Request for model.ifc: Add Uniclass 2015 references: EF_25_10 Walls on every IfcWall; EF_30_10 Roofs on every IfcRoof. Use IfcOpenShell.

First a look at what the model holds.

```python
import ifcopenshell

model = ifcopenshell.open("model.ifc")
print(model.schema)
print("classifications:", [c.Name for c in model.by_type("IfcClassification")])
for ifc_class in ("IfcDoor", "IfcRoof", "IfcStair", "IfcWall", "IfcWindow"):
    print(ifc_class, len(model.by_type(ifc_class)))
```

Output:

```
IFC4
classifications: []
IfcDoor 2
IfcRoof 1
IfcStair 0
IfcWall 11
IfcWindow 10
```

```python
import ifcopenshell
import ifcopenshell.api.classification

model = ifcopenshell.open("model.ifc")

system = ifcopenshell.api.classification.add_classification(model, classification="Uniclass 2015")

codes = {
    "IfcWall": ("EF_25_10", "Walls"),
    "IfcRoof": ("EF_30_10", "Roofs"),
}
for ifc_class, (code, name) in codes.items():
    products = model.by_type(ifc_class)
    ifcopenshell.api.classification.add_reference(
        model, products=products, classification=system, identification=code, name=name
    )
    print(code, len(products))

model.write("model-out.ifc")
```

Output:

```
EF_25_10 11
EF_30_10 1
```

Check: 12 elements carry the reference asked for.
